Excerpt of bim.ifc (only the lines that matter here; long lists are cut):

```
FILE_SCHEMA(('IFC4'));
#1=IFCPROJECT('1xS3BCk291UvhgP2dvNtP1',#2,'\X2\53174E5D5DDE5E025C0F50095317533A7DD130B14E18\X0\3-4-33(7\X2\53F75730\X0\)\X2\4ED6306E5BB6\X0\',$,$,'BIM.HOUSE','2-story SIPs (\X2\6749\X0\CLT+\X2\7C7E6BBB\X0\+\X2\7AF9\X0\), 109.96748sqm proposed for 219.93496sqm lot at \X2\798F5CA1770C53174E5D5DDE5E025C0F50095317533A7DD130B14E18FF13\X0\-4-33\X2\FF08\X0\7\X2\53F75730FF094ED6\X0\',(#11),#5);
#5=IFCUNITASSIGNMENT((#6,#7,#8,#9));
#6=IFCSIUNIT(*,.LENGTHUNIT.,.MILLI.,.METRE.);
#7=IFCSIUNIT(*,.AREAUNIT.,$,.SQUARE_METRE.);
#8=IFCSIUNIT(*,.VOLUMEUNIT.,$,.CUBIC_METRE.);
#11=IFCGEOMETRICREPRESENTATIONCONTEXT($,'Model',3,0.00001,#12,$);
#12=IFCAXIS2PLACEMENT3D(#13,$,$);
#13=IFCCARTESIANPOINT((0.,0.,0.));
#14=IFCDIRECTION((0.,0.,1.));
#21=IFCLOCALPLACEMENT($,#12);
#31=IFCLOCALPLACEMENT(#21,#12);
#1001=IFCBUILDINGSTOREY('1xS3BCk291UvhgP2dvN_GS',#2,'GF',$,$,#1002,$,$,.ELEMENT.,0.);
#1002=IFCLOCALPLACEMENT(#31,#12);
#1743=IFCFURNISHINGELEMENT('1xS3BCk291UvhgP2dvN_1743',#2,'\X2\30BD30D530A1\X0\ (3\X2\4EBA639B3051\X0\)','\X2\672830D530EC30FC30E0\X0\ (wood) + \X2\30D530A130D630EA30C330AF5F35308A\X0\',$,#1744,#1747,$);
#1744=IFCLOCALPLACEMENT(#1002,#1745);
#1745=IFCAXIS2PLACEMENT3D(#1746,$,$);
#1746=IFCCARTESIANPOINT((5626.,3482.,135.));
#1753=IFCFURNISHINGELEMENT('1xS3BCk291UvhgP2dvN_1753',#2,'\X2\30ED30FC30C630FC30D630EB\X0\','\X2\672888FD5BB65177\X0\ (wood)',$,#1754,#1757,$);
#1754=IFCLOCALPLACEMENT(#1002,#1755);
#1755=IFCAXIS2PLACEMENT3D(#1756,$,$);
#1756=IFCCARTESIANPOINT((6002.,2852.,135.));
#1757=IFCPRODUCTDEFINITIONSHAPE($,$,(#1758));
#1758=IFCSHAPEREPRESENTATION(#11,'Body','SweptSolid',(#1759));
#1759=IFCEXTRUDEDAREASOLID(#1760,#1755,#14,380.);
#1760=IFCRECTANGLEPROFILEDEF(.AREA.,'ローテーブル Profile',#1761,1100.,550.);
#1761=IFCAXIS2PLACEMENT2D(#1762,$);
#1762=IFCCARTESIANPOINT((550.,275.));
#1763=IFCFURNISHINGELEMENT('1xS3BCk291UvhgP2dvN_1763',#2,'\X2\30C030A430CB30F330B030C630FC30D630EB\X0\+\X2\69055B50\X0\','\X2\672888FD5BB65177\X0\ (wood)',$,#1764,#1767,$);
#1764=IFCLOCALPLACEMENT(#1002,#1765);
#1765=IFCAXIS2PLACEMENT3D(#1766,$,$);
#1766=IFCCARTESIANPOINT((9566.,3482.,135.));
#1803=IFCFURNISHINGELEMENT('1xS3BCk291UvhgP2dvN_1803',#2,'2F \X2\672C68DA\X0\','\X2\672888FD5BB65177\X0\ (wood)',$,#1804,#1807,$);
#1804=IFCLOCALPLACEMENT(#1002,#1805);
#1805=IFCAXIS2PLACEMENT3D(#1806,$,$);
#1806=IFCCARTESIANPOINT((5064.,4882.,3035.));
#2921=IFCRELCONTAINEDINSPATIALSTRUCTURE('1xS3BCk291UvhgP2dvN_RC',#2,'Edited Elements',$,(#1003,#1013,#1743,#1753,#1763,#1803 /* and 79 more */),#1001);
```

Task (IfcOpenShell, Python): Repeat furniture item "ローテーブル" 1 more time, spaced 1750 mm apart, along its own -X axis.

```python
import ifcopenshell
import ifcopenshell.api.geometry
import ifcopenshell.api.root
import ifcopenshell.util.element
import ifcopenshell.util.placement
import ifcopenshell.util.unit

model = ifcopenshell.open("bim.ifc")
unit_scale = ifcopenshell.util.unit.calculate_unit_scale(model)


def reuse_history(source, copy):
    """copy_class also copies each property set's owner history, people and application; keep the originals."""
    for rel in copy.IsDefinedBy:
        if rel.is_a("IfcRelDefinesByProperties") and (history := rel.RelatingPropertyDefinition.OwnerHistory):
            rel.RelatingPropertyDefinition.OwnerHistory = source.OwnerHistory
            ifcopenshell.util.element.remove_deep2(model, history)


source = model.by_guid("1xS3BCk291UvhgP2dvN_1753")
base = ifcopenshell.util.placement.get_local_placement(source.ObjectPlacement)
step = -base[:3, 0] * 1.75 / unit_scale

for i in range(1, 2):
    copy = ifcopenshell.api.root.copy_class(model, product=source)
    copy.Representation = ifcopenshell.util.element.copy_deep(
        model, source.Representation, exclude=["IfcGeometricRepresentationContext", "IfcRepresentationMap"]
    )
    reuse_history(source, copy)
    matrix = base.copy()
    matrix[:3, 3] += i * step
    print("added at", matrix[:3, 3].round(3) + 0.0)
    ifcopenshell.api.geometry.edit_object_placement(model, product=copy, matrix=matrix, is_si=False)

model.write("bim_rev.ifc")
```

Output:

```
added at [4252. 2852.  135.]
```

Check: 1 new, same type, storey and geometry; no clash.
